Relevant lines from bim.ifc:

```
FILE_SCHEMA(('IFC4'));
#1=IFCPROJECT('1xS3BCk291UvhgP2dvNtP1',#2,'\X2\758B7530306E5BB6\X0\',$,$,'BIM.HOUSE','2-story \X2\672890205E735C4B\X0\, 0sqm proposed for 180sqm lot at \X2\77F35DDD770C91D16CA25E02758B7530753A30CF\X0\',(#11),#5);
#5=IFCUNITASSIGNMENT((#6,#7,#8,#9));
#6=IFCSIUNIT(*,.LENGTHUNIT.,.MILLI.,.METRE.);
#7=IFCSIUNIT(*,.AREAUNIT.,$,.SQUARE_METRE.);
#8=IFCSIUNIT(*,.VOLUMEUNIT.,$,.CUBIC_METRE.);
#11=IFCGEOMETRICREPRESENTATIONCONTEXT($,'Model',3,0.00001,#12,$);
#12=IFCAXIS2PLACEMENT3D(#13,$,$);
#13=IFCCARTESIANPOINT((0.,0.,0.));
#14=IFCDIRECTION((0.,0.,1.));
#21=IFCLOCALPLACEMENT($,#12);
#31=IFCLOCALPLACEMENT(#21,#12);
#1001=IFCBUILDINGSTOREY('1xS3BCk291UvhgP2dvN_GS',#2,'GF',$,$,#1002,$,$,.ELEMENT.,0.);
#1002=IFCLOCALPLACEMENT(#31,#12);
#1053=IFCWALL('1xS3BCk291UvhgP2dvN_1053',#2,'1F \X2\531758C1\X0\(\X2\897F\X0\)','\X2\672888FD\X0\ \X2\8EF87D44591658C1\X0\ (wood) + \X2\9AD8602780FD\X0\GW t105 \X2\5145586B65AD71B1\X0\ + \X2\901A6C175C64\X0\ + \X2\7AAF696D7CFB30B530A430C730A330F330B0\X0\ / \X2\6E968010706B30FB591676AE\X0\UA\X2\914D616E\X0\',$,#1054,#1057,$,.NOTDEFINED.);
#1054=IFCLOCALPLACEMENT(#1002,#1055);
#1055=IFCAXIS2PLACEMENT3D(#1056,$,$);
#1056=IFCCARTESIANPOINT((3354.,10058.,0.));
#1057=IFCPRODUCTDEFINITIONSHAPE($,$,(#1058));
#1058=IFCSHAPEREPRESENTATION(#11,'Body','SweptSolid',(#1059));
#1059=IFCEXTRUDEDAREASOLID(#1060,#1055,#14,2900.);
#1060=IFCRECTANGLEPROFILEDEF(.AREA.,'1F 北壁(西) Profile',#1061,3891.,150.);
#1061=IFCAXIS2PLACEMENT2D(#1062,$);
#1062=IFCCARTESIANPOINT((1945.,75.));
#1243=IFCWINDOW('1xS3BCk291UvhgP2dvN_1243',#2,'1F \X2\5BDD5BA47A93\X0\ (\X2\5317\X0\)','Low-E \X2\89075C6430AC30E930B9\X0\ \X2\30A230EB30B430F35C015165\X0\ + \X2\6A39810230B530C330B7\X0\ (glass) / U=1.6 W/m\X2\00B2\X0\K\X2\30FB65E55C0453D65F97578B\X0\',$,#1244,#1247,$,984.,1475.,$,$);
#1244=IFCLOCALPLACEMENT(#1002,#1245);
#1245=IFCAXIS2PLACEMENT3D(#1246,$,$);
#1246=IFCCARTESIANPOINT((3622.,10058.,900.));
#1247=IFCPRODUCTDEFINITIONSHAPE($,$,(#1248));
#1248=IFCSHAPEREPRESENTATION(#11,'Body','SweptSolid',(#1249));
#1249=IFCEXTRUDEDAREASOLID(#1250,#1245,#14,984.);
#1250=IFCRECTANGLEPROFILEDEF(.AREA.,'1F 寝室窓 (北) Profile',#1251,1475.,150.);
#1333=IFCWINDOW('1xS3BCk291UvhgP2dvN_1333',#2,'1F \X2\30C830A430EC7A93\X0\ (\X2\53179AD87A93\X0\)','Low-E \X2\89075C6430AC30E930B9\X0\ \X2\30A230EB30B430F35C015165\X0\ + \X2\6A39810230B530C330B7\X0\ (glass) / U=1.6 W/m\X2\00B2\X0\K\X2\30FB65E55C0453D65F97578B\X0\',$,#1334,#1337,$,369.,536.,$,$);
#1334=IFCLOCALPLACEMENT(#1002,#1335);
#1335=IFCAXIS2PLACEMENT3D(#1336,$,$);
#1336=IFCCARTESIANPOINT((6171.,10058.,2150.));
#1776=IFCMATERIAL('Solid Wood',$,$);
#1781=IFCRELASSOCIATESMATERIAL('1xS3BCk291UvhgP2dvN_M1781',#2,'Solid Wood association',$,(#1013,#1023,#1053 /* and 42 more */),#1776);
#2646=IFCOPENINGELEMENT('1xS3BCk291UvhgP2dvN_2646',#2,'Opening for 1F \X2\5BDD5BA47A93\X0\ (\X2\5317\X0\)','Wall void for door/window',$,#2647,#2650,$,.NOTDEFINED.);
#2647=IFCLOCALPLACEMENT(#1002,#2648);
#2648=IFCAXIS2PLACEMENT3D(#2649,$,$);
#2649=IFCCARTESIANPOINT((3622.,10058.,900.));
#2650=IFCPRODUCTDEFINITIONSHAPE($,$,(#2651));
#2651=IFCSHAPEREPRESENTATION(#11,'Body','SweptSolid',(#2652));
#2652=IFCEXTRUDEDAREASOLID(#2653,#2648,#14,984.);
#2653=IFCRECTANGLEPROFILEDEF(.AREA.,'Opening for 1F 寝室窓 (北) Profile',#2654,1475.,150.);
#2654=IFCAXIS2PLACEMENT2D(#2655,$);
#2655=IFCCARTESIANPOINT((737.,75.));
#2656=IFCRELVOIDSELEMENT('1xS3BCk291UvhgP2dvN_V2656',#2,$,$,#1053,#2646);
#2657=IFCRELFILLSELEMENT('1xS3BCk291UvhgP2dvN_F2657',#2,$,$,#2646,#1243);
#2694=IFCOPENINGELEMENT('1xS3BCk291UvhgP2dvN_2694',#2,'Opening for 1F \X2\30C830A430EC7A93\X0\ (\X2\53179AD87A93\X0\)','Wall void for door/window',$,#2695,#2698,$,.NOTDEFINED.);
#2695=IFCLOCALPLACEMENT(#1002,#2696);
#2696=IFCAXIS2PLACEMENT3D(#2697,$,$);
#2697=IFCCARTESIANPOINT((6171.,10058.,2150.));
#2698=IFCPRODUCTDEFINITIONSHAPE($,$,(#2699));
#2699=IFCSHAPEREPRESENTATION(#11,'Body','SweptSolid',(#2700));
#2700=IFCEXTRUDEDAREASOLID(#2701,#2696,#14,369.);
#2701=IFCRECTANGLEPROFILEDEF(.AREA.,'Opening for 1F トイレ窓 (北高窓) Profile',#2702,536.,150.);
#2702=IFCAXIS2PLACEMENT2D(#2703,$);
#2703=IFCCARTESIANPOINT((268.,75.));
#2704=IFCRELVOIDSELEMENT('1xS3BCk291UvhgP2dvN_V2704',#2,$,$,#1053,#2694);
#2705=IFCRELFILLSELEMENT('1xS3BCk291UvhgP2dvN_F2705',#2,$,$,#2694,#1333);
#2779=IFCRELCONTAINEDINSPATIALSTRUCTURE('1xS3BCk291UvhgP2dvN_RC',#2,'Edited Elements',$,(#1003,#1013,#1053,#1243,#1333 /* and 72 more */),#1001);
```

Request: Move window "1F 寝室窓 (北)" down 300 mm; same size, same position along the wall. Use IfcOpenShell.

```python
import numpy as np
import ifcopenshell
import ifcopenshell.api.geometry
import ifcopenshell.util.placement
import ifcopenshell.util.unit

model = ifcopenshell.open("bim.ifc")
unit_scale = ifcopenshell.util.unit.calculate_unit_scale(model)

window = model.by_guid("1xS3BCk291UvhgP2dvN_1243")
opening = window.FillsVoids[0].RelatingOpeningElement
dz = -0.3 / unit_scale

shift = np.array([0.0, 0.0, dz])
# The window is not placed relative to its opening, so move both.
for product in (opening, window):
    matrix = ifcopenshell.util.placement.get_local_placement(product.ObjectPlacement)
    matrix[:3, 3] += shift
    ifcopenshell.api.geometry.edit_object_placement(model, product=product, matrix=matrix, is_si=False)

print(f"moved by {dz * unit_scale:+.3f} m")

model.write("bim_v2.ifc")
```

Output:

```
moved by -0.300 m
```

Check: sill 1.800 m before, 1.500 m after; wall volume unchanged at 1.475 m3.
